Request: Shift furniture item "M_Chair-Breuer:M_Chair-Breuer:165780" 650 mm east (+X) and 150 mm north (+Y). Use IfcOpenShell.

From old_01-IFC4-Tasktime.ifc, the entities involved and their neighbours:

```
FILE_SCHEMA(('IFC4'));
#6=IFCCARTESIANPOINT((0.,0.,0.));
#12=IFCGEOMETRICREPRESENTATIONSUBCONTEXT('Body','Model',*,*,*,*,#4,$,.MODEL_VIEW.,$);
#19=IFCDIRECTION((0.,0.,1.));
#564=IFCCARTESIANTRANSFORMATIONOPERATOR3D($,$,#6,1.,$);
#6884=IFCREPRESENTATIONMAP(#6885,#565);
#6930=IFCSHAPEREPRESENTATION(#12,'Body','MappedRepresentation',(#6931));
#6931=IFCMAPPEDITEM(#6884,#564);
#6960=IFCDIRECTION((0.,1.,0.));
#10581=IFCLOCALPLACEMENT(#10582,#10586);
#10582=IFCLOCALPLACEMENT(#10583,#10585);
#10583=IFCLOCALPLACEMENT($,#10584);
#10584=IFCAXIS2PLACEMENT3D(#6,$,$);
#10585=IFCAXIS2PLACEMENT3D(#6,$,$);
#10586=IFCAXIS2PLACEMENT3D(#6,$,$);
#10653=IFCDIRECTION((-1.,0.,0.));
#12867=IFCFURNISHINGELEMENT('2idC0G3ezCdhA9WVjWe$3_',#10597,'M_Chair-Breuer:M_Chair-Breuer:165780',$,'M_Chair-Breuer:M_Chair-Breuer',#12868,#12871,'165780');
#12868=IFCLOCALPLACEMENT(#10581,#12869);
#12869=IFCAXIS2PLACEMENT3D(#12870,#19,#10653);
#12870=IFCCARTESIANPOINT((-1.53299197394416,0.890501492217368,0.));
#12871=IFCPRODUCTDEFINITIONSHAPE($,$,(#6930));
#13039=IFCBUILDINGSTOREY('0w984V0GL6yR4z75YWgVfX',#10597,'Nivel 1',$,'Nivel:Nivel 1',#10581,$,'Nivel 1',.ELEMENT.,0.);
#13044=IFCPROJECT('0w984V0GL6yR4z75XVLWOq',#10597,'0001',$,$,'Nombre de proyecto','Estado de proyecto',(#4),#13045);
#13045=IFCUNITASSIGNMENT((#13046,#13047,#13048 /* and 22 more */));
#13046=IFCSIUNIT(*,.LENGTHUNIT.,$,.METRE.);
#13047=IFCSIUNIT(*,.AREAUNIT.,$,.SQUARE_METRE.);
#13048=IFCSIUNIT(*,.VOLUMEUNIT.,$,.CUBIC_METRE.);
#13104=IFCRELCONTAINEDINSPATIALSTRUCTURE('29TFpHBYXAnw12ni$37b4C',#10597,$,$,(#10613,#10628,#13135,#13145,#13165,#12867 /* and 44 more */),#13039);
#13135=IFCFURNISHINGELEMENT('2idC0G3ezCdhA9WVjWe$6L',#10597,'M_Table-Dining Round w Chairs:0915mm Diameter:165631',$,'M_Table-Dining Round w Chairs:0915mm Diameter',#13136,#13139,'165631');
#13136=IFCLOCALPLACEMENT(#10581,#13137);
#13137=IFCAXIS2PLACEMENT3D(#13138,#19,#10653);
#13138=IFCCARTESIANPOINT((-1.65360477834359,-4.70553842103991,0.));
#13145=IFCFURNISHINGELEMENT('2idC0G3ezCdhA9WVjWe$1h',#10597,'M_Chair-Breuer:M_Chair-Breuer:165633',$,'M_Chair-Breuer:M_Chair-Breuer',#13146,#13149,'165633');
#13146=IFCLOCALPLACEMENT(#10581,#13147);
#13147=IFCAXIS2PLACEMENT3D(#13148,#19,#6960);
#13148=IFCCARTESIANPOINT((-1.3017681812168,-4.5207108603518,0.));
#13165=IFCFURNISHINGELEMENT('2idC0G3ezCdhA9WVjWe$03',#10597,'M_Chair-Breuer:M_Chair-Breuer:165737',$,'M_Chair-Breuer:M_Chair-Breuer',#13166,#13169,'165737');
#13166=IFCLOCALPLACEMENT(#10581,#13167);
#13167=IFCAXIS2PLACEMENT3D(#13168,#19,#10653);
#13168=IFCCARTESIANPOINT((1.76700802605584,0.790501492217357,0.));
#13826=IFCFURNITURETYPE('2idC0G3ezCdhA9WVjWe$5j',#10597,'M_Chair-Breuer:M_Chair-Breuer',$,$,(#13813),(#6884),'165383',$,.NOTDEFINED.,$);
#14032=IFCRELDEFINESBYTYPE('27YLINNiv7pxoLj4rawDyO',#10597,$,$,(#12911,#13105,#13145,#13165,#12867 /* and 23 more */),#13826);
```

```python
import ifcopenshell
import ifcopenshell.api.geometry
import ifcopenshell.util.placement
import ifcopenshell.util.unit

model = ifcopenshell.open("old_01-IFC4-Tasktime.ifc")
unit_scale = ifcopenshell.util.unit.calculate_unit_scale(model)

item = model.by_guid("2idC0G3ezCdhA9WVjWe$3_")
matrix = ifcopenshell.util.placement.get_local_placement(item.ObjectPlacement)
matrix[0, 3] += 0.65 / unit_scale
matrix[1, 3] += 0.15 / unit_scale
ifcopenshell.api.geometry.edit_object_placement(model, product=item, matrix=matrix, is_si=False)

print(ifcopenshell.util.placement.get_local_placement(item.ObjectPlacement).round(3) + 0.0)

model.write("old_01-IFC4-Tasktime_rev.ifc")
```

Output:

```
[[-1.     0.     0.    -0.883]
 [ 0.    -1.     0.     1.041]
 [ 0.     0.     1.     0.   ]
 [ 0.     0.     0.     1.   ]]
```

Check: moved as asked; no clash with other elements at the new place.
